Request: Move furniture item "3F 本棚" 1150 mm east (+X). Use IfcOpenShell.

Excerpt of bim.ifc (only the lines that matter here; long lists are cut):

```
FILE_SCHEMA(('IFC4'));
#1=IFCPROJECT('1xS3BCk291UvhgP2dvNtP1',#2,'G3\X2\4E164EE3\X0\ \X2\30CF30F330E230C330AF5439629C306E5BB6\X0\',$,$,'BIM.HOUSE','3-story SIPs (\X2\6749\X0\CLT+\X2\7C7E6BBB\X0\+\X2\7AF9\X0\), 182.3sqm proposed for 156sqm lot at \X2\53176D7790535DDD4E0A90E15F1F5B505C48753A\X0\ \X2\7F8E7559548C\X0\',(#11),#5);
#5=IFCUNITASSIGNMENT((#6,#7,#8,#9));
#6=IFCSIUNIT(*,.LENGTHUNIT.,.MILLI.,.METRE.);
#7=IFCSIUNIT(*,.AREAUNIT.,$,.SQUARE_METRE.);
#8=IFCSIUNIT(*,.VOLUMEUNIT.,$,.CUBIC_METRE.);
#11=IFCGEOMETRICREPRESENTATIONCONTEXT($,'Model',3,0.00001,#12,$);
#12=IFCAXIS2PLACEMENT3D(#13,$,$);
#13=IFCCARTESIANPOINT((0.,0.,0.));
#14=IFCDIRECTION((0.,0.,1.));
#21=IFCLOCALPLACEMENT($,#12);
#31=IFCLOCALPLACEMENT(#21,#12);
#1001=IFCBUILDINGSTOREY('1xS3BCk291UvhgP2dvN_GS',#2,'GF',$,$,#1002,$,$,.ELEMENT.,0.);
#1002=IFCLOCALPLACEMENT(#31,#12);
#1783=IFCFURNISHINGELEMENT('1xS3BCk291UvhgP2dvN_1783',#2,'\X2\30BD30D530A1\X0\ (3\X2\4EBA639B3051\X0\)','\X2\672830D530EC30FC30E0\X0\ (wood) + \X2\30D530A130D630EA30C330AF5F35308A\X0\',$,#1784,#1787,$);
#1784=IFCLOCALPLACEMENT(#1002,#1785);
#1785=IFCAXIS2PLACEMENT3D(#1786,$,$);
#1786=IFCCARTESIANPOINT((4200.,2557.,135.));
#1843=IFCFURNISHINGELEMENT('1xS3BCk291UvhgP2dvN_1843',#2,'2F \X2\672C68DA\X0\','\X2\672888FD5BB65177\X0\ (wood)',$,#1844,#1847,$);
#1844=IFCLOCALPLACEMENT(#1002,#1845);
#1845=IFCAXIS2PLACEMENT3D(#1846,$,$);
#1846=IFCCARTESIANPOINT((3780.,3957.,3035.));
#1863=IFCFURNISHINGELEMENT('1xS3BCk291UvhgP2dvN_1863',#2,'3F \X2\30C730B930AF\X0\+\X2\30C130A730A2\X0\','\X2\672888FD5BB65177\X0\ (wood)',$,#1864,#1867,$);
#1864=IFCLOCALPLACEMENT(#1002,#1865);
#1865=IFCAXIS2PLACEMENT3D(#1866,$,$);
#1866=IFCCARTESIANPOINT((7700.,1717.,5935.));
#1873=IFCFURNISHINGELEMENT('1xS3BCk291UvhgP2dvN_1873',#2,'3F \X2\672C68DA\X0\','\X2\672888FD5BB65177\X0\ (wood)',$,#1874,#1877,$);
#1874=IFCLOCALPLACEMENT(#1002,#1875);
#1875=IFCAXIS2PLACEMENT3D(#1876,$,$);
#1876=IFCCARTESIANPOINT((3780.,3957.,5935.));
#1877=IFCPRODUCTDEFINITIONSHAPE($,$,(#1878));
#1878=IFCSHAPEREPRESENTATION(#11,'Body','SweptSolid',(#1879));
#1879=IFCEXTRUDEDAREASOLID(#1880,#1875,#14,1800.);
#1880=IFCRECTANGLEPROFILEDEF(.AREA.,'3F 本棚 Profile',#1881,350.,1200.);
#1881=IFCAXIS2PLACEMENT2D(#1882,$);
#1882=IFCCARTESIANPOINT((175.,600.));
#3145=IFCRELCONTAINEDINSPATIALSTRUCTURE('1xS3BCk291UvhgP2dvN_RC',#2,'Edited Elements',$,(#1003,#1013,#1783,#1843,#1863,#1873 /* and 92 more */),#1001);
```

```python
import ifcopenshell
import ifcopenshell.api.geometry
import ifcopenshell.util.placement
import ifcopenshell.util.unit

model = ifcopenshell.open("bim.ifc")
unit_scale = ifcopenshell.util.unit.calculate_unit_scale(model)

item = model.by_id(1873)
matrix = ifcopenshell.util.placement.get_local_placement(item.ObjectPlacement)
matrix[0, 3] += 1.15 / unit_scale
ifcopenshell.api.geometry.edit_object_placement(model, product=item, matrix=matrix, is_si=False)

print(ifcopenshell.util.placement.get_local_placement(item.ObjectPlacement).round(3) + 0.0)

model.write("bim_v2.ifc")
```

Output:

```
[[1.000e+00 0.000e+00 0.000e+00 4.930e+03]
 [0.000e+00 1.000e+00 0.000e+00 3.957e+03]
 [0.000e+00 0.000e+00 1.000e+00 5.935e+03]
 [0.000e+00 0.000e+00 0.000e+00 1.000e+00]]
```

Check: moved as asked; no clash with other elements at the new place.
